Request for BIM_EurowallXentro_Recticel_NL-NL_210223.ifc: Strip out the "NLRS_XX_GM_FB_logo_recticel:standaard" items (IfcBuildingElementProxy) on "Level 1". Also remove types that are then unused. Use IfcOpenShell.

First a look at what the model holds.

```python
import ifcopenshell
import ifcopenshell.util.element

model = ifcopenshell.open("BIM_EurowallXentro_Recticel_NL-NL_210223.ifc")
print(model.schema)
storey = next(s for s in model.by_type("IfcBuildingStorey") if s.Name == "Level 1")
proxies = [e for e in ifcopenshell.util.element.get_decomposition(storey) if e.is_a("IfcBuildingElementProxy")]
seen = {}
for e in proxies:
    element_type = ifcopenshell.util.element.get_type(e)
    name = element_type.Name if element_type not in (None, e) else None
    seen[name] = seen.get(name, 0) + 1
for name, count in sorted(seen.items(), key=str):
    print(count, "x", name)
```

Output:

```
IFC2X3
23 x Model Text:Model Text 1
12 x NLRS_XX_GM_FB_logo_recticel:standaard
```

```python
import ifcopenshell
import ifcopenshell.api.root
import ifcopenshell.util.element

model = ifcopenshell.open("BIM_EurowallXentro_Recticel_NL-NL_210223.ifc")

storey = next(s for s in model.by_type("IfcBuildingStorey") if s.Name == "Level 1")
proxies = [e for e in ifcopenshell.util.element.get_decomposition(storey) if e.is_a("IfcBuildingElementProxy")]
targets = [e for e in proxies if (t := ifcopenshell.util.element.get_type(e)) not in (None, e) and t.Name == "NLRS_XX_GM_FB_logo_recticel:standaard"]
types = {ifcopenshell.util.element.get_type(e) for e in targets} - {None, *targets}

for e in targets:
    ifcopenshell.api.root.remove_product(model, product=e)
print(len(targets), "removed")

unused = [t for t in types if not ifcopenshell.util.element.get_types(t)]
for t in unused:
    ifcopenshell.api.root.remove_product(model, product=t)
print(len(unused), "unused types removed")

model.write("BIM_EurowallXentro_Recticel_NL-NL_210223_rev.ifc")
```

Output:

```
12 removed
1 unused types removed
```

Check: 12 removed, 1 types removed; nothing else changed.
